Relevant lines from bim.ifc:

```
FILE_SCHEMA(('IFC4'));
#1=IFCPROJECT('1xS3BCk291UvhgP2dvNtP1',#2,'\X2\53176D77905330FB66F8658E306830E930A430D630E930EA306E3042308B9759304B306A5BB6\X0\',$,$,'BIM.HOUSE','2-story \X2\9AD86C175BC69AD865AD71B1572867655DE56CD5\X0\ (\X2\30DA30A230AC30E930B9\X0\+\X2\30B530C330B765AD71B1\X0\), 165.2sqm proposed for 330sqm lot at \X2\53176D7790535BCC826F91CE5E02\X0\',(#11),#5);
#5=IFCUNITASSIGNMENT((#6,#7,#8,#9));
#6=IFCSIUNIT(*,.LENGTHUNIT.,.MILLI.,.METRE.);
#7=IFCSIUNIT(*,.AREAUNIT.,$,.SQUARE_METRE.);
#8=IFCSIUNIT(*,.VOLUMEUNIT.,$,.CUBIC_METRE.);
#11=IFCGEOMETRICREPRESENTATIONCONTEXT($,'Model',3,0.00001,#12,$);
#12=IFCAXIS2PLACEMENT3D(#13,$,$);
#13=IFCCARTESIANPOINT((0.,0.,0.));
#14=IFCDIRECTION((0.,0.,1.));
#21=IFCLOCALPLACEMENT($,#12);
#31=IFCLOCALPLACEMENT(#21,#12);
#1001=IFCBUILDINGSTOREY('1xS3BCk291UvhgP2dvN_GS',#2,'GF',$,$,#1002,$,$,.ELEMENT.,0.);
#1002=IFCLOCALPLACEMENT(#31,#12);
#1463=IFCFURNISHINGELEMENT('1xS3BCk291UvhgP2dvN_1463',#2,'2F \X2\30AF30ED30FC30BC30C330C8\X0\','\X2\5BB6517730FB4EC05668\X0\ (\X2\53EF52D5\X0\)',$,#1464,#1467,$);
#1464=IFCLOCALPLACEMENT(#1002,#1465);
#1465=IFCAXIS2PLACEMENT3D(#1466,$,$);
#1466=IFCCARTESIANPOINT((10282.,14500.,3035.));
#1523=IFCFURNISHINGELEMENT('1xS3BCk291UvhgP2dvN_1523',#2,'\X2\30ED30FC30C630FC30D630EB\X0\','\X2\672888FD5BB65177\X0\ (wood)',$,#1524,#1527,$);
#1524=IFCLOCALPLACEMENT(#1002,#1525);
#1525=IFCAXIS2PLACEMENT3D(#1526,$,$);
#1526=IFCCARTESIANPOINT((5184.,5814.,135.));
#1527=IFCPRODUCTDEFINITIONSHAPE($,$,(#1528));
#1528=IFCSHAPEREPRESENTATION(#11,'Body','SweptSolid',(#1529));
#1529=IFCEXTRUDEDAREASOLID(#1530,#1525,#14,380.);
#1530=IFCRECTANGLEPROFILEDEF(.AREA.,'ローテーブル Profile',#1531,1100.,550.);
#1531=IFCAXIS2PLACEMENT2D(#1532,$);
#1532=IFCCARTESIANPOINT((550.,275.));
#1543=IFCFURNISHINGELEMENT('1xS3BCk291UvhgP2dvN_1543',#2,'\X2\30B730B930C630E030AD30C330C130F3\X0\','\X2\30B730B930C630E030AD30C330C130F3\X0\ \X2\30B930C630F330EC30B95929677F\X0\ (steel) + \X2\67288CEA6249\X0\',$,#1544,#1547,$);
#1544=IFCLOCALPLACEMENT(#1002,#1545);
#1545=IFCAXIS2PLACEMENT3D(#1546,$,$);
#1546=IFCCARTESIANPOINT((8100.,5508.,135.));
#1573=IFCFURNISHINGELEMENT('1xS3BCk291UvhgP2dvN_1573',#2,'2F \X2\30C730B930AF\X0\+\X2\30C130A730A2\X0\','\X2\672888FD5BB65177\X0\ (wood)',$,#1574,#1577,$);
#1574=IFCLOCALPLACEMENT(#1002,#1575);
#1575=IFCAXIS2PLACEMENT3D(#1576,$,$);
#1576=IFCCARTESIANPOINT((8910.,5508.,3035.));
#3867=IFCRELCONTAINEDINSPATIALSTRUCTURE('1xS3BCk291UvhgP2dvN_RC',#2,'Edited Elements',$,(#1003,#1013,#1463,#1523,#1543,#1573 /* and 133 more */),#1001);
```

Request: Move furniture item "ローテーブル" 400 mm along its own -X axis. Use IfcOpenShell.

```python
import ifcopenshell
import ifcopenshell.api.geometry
import ifcopenshell.util.placement

model = ifcopenshell.open("bim.ifc")

item = model.by_id(1523)
matrix = ifcopenshell.util.placement.get_local_placement(item.ObjectPlacement)
matrix[:3, 3] -= matrix[:3, 0] * 400.0
ifcopenshell.api.geometry.edit_object_placement(model, product=item, matrix=matrix, is_si=False)

print(ifcopenshell.util.placement.get_local_placement(item.ObjectPlacement).round(3) + 0.0)

model.write("bim_rev.ifc")
```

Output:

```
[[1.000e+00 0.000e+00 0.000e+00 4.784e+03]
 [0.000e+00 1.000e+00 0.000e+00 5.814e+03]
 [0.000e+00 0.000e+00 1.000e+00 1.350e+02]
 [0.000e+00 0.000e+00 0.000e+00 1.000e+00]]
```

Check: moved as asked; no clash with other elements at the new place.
